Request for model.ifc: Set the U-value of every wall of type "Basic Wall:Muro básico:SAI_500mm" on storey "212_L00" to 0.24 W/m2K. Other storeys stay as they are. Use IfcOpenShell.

First a look at what the model holds.

```python
import ifcopenshell
import ifcopenshell.util.element

model = ifcopenshell.open("model.ifc")
print(model.schema)
storey = next(s for s in model.by_type("IfcBuildingStorey") if s.Name == "212_L00")
walls = [e for e in ifcopenshell.util.element.get_decomposition(storey) if e.is_a("IfcWall")]
seen = {}
for e in walls:
    element_type = ifcopenshell.util.element.get_type(e)
    key = (element_type.Name if element_type != e and element_type else None, ifcopenshell.util.element.get_pset(e, "Pset_WallCommon", "ThermalTransmittance"))
    seen[key] = seen.get(key, 0) + 1
for (name, value), count in sorted(seen.items(), key=str):
    print(count, "x", name, "|", value)
```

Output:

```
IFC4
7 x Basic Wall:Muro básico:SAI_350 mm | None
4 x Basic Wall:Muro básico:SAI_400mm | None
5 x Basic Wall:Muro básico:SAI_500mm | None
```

```python
import ifcopenshell
import ifcopenshell.api.pset
import ifcopenshell.util.element

model = ifcopenshell.open("model.ifc")

storey = next(s for s in model.by_type("IfcBuildingStorey") if s.Name == "212_L00")
walls = [e for e in ifcopenshell.util.element.get_decomposition(storey) if e.is_a("IfcWall")]

count = 0
for e in walls:
    element_type = ifcopenshell.util.element.get_type(e)
    if element_type in (None, e) or element_type.Name != "Basic Wall:Muro básico:SAI_500mm":
        continue
    # add_pset returns the element's existing set when there is one.
    pset = ifcopenshell.api.pset.add_pset(model, product=e, name="Pset_WallCommon")
    ifcopenshell.api.pset.edit_pset(model, pset=pset, properties={"ThermalTransmittance": 0.24})
    count += 1

print(count, "walls updated")

model.write("model_v2.ifc")
```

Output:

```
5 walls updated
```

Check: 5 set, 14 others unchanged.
